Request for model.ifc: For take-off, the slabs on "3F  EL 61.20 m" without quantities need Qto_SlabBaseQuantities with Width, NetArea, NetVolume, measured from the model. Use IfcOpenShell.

First a look at what the model holds.

```python
import ifcopenshell
import ifcopenshell.util.element
import ifcopenshell.util.unit

model = ifcopenshell.open("model.ifc")
print(model.schema)
for unit_type in ("LENGTHUNIT", "AREAUNIT", "VOLUMEUNIT"):
    print(unit_type, ifcopenshell.util.unit.calculate_unit_scale(model, unit_type))
storey = next(s for s in model.by_type("IfcBuildingStorey") if s.Name == "3F  EL 61.20 m")
slabs = [e for e in ifcopenshell.util.element.get_decomposition(storey) if e.is_a("IfcSlab")]
for e in sorted(slabs, key=lambda e: e.id()):
    print(e.id(), e.is_a(), e.Name, list(ifcopenshell.util.element.get_psets(e, qtos_only=True)), sep=" | ")
```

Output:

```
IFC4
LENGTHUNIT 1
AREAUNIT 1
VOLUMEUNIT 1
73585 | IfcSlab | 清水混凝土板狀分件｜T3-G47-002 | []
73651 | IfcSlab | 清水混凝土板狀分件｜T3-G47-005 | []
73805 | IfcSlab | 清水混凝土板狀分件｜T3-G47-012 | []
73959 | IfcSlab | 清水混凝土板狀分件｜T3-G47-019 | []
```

```python
import ifcopenshell
import ifcopenshell.api.pset
import ifcopenshell.geom
import ifcopenshell.util.element
import ifcopenshell.util.shape
import ifcopenshell.util.unit

model = ifcopenshell.open("model.ifc")
unit_scale = ifcopenshell.util.unit.calculate_unit_scale(model)
area_scale = ifcopenshell.util.unit.calculate_unit_scale(model, "AREAUNIT")
volume_scale = ifcopenshell.util.unit.calculate_unit_scale(model, "VOLUMEUNIT")
settings = ifcopenshell.geom.settings()

storey = next(s for s in model.by_type("IfcBuildingStorey") if s.Name == "3F  EL 61.20 m")
slabs = [e for e in ifcopenshell.util.element.get_decomposition(storey) if e.is_a("IfcSlab")]

for e in sorted(slabs, key=lambda e: e.id()):
    if ifcopenshell.util.element.get_psets(e, qtos_only=True, should_inherit=False):
        continue
    # Geometry comes back in metres, in the element's own axes.
    shape = ifcopenshell.geom.create_shape(settings, e)
    values = {
        "Width": ifcopenshell.util.shape.get_z(shape.geometry) / unit_scale,
        "NetArea": ifcopenshell.util.shape.get_footprint_area(shape.geometry) / area_scale,
        "NetVolume": ifcopenshell.util.shape.get_volume(shape.geometry) / volume_scale,
    }
    qto = ifcopenshell.api.pset.add_qto(model, product=e, name="Qto_SlabBaseQuantities")
    ifcopenshell.api.pset.edit_qto(model, qto=qto, properties=values)
    print(e.id(), {k: round(v, 3) for k, v in values.items()})

model.write("model-out.ifc")
```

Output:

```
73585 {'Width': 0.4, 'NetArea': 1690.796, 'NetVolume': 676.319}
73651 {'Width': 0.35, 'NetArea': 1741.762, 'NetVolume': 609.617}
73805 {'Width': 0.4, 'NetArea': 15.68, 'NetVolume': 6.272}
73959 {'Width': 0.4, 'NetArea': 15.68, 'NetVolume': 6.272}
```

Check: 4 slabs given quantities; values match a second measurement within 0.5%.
